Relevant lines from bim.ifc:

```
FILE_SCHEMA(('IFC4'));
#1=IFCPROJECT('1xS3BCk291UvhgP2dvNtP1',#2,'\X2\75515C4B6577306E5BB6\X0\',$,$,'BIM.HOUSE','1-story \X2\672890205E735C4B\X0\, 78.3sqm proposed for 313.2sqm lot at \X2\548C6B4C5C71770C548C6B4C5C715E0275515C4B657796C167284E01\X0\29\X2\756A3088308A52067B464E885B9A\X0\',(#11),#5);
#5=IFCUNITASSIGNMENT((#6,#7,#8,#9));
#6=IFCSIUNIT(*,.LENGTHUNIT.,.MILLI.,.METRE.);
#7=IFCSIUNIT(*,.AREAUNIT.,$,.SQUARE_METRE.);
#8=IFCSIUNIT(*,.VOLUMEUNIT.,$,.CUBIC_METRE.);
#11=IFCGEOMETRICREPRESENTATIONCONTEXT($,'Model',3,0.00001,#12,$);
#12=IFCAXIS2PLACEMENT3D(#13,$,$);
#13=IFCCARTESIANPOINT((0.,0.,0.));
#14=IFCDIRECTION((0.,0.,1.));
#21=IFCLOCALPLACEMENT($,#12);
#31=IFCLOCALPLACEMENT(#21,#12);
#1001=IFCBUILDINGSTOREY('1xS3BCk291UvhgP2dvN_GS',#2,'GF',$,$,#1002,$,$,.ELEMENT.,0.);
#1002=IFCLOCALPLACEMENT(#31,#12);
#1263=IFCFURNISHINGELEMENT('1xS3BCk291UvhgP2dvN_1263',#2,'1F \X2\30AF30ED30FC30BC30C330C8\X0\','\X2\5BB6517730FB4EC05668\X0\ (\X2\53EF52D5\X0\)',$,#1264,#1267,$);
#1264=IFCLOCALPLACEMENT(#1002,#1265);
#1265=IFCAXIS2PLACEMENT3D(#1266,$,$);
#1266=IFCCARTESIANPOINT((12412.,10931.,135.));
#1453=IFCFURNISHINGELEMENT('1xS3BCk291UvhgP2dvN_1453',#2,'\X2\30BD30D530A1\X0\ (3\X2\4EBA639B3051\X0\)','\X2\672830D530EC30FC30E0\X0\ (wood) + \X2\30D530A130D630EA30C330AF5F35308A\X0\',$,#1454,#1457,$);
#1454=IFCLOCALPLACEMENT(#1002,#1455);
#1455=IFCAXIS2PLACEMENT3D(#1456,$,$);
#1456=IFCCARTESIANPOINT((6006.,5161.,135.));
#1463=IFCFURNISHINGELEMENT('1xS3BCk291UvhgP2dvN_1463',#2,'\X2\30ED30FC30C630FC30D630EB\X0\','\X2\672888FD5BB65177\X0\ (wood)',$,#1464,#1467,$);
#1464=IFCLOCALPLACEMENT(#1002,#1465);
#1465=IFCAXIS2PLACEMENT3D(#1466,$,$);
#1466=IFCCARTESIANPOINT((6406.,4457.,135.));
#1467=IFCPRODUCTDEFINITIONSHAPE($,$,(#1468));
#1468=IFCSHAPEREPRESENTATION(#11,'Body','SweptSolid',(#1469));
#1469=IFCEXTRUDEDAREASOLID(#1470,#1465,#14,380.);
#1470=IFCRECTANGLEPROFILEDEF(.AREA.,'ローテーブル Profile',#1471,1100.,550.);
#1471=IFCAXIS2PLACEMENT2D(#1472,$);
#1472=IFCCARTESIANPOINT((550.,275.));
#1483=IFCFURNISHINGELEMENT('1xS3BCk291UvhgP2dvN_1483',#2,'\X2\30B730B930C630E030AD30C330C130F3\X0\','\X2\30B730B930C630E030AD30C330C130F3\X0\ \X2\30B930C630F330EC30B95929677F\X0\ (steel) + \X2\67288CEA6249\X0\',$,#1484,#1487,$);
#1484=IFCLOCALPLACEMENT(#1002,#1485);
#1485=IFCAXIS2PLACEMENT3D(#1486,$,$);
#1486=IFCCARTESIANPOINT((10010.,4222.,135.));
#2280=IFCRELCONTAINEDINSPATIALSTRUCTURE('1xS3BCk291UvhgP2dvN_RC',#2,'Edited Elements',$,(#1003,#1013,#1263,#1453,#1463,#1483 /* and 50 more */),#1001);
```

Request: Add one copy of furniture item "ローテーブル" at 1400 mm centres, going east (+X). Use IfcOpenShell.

```python
import numpy as np
import ifcopenshell
import ifcopenshell.api.geometry
import ifcopenshell.api.root
import ifcopenshell.util.element
import ifcopenshell.util.placement

model = ifcopenshell.open("bim.ifc")


def reuse_history(source, copy):
    """copy_class also copies each property set's owner history, people and application; keep the originals."""
    for rel in copy.IsDefinedBy:
        if rel.is_a("IfcRelDefinesByProperties") and (history := rel.RelatingPropertyDefinition.OwnerHistory):
            rel.RelatingPropertyDefinition.OwnerHistory = source.OwnerHistory
            ifcopenshell.util.element.remove_deep2(model, history)


source = model.by_id(1463)
base = ifcopenshell.util.placement.get_local_placement(source.ObjectPlacement)
step = np.array([1.0, 0.0, 0.0]) * 1400.0

for i in range(1, 2):
    copy = ifcopenshell.api.root.copy_class(model, product=source)
    copy.Representation = ifcopenshell.util.element.copy_deep(
        model, source.Representation, exclude=["IfcGeometricRepresentationContext", "IfcRepresentationMap"]
    )
    reuse_history(source, copy)
    matrix = base.copy()
    matrix[:3, 3] += i * step
    print("added at", matrix[:3, 3].round(3) + 0.0)
    ifcopenshell.api.geometry.edit_object_placement(model, product=copy, matrix=matrix, is_si=False)

model.write("bim_v2.ifc")
```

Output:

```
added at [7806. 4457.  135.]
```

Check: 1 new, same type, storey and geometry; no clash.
